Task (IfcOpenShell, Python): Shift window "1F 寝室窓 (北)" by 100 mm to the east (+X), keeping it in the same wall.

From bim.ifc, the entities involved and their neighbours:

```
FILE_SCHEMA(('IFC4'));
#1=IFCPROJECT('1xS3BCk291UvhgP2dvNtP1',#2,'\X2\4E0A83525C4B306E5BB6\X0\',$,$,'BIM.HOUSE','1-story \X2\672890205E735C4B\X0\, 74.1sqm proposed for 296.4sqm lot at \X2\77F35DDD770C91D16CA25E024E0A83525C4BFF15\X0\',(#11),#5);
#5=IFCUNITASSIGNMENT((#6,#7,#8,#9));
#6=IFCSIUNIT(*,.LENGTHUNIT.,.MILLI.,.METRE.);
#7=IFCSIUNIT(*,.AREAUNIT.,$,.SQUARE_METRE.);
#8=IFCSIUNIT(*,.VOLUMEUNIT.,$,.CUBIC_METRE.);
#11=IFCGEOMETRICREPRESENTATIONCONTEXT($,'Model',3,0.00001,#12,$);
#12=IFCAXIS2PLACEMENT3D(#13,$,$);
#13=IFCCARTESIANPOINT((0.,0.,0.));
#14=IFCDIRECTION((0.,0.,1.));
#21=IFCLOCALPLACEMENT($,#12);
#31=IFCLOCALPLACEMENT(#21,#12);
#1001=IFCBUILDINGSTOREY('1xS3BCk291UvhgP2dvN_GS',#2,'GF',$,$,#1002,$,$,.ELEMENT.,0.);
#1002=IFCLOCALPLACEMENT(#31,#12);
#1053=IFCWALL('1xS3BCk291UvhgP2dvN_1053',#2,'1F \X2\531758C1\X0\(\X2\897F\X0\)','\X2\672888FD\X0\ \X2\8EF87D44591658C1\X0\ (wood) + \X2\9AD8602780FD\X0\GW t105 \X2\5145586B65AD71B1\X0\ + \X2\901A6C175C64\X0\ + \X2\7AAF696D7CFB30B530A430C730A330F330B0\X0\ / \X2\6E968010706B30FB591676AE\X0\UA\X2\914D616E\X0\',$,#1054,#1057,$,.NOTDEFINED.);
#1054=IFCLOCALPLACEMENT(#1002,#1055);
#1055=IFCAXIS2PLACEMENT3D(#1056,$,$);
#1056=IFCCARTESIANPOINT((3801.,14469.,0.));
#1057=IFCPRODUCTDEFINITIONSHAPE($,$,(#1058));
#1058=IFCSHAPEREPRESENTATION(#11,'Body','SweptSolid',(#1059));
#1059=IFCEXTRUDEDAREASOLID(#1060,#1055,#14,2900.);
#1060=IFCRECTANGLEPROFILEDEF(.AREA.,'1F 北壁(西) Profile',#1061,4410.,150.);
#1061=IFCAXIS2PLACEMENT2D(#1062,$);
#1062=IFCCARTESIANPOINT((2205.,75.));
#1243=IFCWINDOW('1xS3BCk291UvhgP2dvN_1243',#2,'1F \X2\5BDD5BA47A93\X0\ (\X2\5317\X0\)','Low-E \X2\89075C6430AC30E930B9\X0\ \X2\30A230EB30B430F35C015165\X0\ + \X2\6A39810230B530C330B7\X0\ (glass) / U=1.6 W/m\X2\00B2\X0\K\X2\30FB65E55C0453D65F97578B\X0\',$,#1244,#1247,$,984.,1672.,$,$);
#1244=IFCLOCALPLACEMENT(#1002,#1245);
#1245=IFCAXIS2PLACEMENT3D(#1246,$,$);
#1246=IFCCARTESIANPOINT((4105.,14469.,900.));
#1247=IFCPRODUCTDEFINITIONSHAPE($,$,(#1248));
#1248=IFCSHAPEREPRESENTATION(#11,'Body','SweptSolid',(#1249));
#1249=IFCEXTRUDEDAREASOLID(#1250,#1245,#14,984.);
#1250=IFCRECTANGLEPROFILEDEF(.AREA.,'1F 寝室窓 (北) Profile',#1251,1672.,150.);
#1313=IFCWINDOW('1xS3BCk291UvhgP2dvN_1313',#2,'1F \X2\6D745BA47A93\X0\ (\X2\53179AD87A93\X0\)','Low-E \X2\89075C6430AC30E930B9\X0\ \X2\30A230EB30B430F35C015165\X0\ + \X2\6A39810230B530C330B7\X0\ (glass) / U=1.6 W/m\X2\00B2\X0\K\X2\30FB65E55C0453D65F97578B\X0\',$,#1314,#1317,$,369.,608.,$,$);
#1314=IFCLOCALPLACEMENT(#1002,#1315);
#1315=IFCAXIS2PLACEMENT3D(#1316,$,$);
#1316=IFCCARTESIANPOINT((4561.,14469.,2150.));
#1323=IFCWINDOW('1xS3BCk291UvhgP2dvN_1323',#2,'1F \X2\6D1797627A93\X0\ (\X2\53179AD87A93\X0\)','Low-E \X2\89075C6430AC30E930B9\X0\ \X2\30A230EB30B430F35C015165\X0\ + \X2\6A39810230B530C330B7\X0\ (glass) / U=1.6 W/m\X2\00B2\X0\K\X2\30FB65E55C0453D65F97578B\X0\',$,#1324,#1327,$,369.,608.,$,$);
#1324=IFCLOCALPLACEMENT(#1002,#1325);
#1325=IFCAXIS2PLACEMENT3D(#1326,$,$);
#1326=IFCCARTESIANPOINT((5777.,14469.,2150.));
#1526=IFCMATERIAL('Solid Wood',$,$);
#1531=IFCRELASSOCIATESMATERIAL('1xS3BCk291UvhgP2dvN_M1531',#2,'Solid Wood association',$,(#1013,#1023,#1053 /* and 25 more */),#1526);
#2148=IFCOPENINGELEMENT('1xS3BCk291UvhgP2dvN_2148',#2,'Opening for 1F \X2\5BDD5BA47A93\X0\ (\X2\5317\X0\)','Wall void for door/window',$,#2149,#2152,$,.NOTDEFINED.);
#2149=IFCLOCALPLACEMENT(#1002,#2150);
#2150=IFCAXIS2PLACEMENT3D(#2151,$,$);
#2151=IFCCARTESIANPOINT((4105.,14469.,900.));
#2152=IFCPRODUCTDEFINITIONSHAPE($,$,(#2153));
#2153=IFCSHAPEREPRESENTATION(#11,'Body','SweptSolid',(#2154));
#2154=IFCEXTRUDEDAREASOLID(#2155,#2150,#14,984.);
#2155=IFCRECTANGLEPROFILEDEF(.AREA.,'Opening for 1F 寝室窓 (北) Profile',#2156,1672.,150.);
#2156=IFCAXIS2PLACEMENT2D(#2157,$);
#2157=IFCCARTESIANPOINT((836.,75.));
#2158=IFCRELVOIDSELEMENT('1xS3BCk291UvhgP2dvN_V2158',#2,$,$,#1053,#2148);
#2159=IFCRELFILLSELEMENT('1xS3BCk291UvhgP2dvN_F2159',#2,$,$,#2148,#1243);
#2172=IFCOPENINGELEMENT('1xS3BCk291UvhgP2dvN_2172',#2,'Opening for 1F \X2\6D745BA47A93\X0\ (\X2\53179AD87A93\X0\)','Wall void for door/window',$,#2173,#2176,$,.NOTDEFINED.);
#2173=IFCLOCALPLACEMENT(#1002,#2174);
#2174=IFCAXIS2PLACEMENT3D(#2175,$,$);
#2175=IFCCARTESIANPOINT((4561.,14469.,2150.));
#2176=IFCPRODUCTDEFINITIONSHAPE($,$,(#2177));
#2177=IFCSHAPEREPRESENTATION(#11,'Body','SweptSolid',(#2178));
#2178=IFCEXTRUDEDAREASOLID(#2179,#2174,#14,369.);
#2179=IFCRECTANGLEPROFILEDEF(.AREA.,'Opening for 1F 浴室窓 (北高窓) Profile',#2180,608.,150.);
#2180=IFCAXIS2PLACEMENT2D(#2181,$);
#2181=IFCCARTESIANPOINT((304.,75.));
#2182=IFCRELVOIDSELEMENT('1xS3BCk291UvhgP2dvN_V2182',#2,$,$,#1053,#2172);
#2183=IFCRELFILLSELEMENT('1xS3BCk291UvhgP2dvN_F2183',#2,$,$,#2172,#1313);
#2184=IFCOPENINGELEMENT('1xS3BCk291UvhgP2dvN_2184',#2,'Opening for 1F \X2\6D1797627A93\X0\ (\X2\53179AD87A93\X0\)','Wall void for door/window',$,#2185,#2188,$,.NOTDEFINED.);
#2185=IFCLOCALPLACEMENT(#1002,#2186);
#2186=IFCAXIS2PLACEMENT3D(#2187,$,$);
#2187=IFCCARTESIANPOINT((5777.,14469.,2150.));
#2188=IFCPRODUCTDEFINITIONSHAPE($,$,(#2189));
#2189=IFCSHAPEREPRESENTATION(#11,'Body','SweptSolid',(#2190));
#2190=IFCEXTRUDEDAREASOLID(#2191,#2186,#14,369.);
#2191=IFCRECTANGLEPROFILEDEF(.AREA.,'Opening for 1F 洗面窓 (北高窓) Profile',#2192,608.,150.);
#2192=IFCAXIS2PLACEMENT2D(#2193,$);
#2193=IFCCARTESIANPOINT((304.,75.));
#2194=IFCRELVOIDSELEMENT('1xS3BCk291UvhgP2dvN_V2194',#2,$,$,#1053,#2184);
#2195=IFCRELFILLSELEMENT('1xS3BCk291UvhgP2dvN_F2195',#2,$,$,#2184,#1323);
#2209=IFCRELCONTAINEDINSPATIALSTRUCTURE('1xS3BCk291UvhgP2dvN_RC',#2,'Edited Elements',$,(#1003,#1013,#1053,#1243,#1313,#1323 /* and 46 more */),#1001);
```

```python
import ifcopenshell
import ifcopenshell.api.geometry
import ifcopenshell.util.placement
import ifcopenshell.util.unit

model = ifcopenshell.open("bim.ifc")
unit_scale = ifcopenshell.util.unit.calculate_unit_scale(model)

window = model.by_id(1243)
opening = window.FillsVoids[0].RelatingOpeningElement
wall = opening.VoidsElements[0].RelatingBuildingElement

wall_matrix = ifcopenshell.util.placement.get_local_placement(wall.ObjectPlacement)
shift = wall_matrix[:3, 0] * 0.1 / unit_scale
before = ifcopenshell.util.placement.get_local_placement(window.ObjectPlacement)[:3, 3].copy()

# The window is not placed relative to its opening, so move both.
for product in (opening, window):
    matrix = ifcopenshell.util.placement.get_local_placement(product.ObjectPlacement)
    matrix[:3, 3] += shift
    ifcopenshell.api.geometry.edit_object_placement(model, product=product, matrix=matrix, is_si=False)

after = ifcopenshell.util.placement.get_local_placement(window.ObjectPlacement)[:3, 3]
print("window moved by", (after - before).round(3) + 0.0)

model.write("bim_rev.ifc")
```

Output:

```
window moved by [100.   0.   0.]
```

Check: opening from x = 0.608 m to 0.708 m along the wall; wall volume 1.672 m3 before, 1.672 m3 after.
